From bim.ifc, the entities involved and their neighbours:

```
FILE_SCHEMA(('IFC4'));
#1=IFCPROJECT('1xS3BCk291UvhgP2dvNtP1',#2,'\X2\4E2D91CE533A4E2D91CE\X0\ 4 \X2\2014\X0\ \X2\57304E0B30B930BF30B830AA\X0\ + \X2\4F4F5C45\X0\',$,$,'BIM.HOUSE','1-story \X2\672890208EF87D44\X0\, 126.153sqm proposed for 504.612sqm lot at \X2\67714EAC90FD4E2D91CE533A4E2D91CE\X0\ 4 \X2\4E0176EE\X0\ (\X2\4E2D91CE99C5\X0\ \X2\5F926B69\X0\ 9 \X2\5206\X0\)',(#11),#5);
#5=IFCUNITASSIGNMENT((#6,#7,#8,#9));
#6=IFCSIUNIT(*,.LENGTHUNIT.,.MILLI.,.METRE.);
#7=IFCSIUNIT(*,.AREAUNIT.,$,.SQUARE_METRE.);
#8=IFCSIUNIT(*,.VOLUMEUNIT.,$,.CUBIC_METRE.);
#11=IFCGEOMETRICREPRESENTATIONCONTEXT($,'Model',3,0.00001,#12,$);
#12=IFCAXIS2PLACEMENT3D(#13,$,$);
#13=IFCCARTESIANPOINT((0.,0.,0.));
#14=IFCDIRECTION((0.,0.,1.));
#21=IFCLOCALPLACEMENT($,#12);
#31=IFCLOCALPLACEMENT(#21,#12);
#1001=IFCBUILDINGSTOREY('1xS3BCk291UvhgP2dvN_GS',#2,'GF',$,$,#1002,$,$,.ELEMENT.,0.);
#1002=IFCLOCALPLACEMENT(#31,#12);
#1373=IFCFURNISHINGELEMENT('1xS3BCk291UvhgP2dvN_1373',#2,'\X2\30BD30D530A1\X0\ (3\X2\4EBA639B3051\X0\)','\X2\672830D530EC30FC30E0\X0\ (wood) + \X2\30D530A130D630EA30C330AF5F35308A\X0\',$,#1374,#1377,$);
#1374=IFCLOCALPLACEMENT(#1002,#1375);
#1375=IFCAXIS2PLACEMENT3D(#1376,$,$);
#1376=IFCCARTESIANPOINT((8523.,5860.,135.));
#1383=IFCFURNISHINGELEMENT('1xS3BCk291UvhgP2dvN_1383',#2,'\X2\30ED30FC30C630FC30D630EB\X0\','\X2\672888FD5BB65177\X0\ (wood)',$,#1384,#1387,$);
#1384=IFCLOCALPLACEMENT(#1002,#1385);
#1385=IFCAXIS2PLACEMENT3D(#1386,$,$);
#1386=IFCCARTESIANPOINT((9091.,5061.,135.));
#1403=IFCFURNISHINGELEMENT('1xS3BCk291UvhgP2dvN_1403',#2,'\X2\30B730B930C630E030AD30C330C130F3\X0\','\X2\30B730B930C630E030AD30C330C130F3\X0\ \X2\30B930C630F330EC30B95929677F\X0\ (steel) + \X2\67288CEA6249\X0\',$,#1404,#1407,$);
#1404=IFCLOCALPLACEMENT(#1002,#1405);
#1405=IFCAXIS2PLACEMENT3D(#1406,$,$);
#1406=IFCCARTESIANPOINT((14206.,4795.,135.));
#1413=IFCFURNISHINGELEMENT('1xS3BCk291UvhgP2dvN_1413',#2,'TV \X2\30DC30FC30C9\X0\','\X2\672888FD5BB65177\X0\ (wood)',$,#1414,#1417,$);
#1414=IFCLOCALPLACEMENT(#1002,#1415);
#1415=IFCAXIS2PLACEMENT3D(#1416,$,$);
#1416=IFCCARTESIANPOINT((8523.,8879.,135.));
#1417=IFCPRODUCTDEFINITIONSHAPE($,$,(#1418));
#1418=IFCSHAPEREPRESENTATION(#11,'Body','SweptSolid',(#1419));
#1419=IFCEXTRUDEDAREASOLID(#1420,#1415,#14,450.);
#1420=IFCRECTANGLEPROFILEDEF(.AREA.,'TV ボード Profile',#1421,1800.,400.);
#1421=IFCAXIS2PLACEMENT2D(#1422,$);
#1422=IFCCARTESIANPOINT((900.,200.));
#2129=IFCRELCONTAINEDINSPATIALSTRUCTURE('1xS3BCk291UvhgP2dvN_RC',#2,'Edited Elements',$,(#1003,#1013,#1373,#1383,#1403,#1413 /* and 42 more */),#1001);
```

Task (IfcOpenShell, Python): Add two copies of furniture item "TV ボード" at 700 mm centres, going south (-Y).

```python
import numpy as np
import ifcopenshell
import ifcopenshell.api.geometry
import ifcopenshell.api.root
import ifcopenshell.util.element
import ifcopenshell.util.placement
import ifcopenshell.util.unit

model = ifcopenshell.open("bim.ifc")
unit_scale = ifcopenshell.util.unit.calculate_unit_scale(model)


def reuse_history(source, copy):
    """copy_class also copies each property set's owner history, people and application; keep the originals."""
    for rel in copy.IsDefinedBy:
        if rel.is_a("IfcRelDefinesByProperties") and (history := rel.RelatingPropertyDefinition.OwnerHistory):
            rel.RelatingPropertyDefinition.OwnerHistory = source.OwnerHistory
            ifcopenshell.util.element.remove_deep2(model, history)


source = model.by_guid("1xS3BCk291UvhgP2dvN_1413")
base = ifcopenshell.util.placement.get_local_placement(source.ObjectPlacement)
step = np.array([0.0, -1.0, 0.0]) * 0.7 / unit_scale

for i in range(1, 3):
    copy = ifcopenshell.api.root.copy_class(model, product=source)
    copy.Representation = ifcopenshell.util.element.copy_deep(
        model, source.Representation, exclude=["IfcGeometricRepresentationContext", "IfcRepresentationMap"]
    )
    reuse_history(source, copy)
    matrix = base.copy()
    matrix[:3, 3] += i * step
    print("added at", matrix[:3, 3].round(3) + 0.0)
    ifcopenshell.api.geometry.edit_object_placement(model, product=copy, matrix=matrix, is_si=False)

model.write("bim-out.ifc")
```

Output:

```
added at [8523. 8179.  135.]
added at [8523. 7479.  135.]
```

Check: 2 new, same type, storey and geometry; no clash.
